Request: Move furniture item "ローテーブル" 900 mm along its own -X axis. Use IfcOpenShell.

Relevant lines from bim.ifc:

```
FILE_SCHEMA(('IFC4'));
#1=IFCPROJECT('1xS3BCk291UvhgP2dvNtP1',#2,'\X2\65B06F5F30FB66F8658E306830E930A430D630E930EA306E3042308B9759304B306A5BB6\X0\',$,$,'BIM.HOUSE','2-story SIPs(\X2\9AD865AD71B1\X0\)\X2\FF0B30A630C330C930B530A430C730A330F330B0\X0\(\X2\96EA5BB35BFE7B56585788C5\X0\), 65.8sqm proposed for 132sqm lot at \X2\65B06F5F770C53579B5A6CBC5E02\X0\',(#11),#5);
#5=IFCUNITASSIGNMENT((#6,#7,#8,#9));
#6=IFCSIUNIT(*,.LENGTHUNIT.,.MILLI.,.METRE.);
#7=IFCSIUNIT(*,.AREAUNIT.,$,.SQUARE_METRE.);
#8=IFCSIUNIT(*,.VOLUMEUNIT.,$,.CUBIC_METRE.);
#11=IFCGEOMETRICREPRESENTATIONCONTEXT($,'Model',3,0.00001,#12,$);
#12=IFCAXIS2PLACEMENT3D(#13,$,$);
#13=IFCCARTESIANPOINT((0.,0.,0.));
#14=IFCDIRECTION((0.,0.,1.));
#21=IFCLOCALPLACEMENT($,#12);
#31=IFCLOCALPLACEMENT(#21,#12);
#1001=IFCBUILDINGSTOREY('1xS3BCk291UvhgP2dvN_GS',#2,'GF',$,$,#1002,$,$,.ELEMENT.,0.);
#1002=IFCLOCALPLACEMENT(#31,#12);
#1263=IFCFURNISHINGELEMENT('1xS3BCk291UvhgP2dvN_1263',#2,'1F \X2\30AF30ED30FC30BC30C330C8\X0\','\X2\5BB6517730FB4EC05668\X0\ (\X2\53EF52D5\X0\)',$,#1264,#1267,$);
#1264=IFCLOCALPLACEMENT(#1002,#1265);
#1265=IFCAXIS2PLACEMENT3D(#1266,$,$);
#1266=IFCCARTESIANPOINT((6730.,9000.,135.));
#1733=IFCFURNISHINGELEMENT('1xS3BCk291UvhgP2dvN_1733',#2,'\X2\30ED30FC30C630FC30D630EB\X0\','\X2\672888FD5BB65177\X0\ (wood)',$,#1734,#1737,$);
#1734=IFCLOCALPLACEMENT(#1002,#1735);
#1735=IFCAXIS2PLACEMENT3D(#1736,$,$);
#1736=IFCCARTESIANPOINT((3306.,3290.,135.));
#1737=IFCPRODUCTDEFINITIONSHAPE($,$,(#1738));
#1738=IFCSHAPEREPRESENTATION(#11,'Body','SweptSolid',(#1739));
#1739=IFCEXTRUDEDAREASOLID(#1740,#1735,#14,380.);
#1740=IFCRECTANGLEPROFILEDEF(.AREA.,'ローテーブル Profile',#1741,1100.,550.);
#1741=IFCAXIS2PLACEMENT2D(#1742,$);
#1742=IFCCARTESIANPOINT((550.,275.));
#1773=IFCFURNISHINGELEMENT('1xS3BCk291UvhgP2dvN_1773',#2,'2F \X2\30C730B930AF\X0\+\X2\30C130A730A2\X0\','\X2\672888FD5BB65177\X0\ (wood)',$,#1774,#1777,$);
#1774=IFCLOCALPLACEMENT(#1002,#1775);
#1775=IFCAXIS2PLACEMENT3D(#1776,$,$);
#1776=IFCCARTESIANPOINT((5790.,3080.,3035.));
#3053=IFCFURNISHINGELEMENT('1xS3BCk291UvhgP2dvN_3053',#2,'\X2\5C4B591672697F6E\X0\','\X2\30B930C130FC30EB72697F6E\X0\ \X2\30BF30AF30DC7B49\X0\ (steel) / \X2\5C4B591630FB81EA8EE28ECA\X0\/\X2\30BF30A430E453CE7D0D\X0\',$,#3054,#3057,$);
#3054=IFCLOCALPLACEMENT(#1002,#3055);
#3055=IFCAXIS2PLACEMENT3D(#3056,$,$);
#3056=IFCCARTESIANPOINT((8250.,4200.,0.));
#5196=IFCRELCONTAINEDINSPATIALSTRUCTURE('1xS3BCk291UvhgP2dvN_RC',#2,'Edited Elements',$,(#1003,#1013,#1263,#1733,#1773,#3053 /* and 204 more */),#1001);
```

```python
import ifcopenshell
import ifcopenshell.api.geometry
import ifcopenshell.util.placement

model = ifcopenshell.open("bim.ifc")

item = model.by_id(1733)
matrix = ifcopenshell.util.placement.get_local_placement(item.ObjectPlacement)
matrix[:3, 3] -= matrix[:3, 0] * 900.0
ifcopenshell.api.geometry.edit_object_placement(model, product=item, matrix=matrix, is_si=False)

print(ifcopenshell.util.placement.get_local_placement(item.ObjectPlacement).round(3) + 0.0)

model.write("bim_updated.ifc")
```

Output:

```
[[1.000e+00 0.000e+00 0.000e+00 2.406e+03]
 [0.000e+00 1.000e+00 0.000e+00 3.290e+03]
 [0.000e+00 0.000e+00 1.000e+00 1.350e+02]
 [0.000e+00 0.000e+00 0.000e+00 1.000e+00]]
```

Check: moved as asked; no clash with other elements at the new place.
